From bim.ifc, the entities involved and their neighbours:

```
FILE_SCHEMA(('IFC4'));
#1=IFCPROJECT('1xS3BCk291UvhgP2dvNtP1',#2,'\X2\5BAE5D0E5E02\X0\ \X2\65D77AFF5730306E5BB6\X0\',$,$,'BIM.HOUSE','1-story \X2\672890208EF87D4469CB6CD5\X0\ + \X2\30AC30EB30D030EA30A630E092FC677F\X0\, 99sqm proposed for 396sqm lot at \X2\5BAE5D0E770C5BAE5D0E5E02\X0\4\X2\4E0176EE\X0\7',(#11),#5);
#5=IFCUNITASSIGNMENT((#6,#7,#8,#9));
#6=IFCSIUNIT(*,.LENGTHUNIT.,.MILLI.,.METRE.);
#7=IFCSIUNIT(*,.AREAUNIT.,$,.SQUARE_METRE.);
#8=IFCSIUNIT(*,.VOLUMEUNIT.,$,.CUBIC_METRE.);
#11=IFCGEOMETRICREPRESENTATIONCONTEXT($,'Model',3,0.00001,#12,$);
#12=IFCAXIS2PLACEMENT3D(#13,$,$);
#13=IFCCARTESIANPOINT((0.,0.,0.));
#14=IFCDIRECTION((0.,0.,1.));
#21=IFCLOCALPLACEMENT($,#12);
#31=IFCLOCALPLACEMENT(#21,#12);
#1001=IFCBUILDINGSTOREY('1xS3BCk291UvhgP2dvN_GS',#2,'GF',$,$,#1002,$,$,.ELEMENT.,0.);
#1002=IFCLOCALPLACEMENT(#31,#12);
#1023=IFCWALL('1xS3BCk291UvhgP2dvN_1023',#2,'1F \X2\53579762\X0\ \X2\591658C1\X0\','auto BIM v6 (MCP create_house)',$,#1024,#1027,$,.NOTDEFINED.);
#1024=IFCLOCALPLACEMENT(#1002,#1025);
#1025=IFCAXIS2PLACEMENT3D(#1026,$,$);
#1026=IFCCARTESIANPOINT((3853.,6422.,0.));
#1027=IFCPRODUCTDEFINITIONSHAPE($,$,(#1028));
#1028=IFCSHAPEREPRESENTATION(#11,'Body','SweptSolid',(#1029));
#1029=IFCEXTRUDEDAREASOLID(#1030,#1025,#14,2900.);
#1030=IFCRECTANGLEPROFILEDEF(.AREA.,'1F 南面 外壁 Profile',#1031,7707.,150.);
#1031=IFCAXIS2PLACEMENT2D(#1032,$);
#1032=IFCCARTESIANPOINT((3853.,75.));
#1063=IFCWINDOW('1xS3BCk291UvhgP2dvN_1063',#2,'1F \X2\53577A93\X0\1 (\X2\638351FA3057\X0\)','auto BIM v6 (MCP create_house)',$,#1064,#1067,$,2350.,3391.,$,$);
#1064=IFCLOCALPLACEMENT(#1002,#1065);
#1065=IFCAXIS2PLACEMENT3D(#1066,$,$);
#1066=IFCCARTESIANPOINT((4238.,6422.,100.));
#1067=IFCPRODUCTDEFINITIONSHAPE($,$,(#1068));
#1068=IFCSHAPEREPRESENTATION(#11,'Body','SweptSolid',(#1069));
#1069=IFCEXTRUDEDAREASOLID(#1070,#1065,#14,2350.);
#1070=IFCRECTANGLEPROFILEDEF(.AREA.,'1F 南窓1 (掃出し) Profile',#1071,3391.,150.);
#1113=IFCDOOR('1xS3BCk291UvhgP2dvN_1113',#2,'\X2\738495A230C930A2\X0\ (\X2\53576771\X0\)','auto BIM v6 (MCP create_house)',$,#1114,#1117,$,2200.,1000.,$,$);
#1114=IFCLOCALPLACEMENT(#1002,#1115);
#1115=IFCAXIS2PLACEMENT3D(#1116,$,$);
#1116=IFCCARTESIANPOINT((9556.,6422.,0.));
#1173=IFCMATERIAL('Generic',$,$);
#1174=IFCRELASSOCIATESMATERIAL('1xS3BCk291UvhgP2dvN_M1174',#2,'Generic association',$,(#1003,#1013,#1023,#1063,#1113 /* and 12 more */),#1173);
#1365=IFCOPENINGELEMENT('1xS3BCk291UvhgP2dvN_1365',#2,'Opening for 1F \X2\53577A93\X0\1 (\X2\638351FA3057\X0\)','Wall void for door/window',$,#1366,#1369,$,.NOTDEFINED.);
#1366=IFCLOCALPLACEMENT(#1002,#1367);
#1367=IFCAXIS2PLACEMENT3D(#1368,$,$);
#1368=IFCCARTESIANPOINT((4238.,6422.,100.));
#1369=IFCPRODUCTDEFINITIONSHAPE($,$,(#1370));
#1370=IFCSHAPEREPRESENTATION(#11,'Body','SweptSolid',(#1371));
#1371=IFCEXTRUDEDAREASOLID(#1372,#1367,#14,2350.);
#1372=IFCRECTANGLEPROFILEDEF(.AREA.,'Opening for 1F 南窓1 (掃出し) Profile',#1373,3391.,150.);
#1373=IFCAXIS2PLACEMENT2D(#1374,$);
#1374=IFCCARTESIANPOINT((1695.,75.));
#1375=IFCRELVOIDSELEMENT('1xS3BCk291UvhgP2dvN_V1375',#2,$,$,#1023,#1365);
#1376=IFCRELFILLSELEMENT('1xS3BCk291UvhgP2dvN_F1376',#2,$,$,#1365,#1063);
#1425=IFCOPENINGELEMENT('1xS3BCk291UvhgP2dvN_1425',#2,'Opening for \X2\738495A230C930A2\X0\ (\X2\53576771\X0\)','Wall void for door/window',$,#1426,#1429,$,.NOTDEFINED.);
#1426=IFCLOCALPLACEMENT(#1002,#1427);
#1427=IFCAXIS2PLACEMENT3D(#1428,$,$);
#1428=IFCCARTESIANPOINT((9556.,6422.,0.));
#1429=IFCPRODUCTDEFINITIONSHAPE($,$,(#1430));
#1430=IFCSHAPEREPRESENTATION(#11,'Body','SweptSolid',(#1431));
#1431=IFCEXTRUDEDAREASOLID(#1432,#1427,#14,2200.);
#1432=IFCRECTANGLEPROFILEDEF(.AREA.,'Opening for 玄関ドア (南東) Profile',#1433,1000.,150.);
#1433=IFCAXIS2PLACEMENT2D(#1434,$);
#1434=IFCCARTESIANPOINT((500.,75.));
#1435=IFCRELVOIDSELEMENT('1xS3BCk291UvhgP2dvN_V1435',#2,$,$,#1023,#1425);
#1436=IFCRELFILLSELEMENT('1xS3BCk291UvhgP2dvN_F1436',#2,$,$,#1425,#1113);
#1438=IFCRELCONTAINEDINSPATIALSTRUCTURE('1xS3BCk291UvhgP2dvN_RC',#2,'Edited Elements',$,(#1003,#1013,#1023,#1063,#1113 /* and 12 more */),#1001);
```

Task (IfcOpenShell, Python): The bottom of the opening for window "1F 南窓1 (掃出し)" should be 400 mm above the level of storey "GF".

```python
import numpy as np
import ifcopenshell
import ifcopenshell.api.geometry
import ifcopenshell.geom
import ifcopenshell.util.element
import ifcopenshell.util.placement
import ifcopenshell.util.shape
import ifcopenshell.util.unit

model = ifcopenshell.open("bim.ifc")
unit_scale = ifcopenshell.util.unit.calculate_unit_scale(model)

window = model.by_id(1063)
opening = window.FillsVoids[0].RelatingOpeningElement
storey = ifcopenshell.util.element.get_container(window, ifc_class="IfcBuildingStorey")
level = ifcopenshell.util.placement.get_local_placement(storey.ObjectPlacement)[2, 3]

# The opening's origin need not be at the sill, so measure its lowest point.
shape = ifcopenshell.geom.create_shape(ifcopenshell.geom.settings(), opening)
bottom = ifcopenshell.util.shape.get_shape_bottom_elevation(shape, shape.geometry) / unit_scale
dz = level + 0.4 / unit_scale - bottom

shift = np.array([0.0, 0.0, dz])
# The window is not placed relative to its opening, so move both.
for product in (opening, window):
    matrix = ifcopenshell.util.placement.get_local_placement(product.ObjectPlacement)
    matrix[:3, 3] += shift
    ifcopenshell.api.geometry.edit_object_placement(model, product=product, matrix=matrix, is_si=False)

print(f"moved by {dz * unit_scale:+.3f} m")

model.write("bim_v2.ifc")
```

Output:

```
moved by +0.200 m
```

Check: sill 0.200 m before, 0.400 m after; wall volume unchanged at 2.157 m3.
